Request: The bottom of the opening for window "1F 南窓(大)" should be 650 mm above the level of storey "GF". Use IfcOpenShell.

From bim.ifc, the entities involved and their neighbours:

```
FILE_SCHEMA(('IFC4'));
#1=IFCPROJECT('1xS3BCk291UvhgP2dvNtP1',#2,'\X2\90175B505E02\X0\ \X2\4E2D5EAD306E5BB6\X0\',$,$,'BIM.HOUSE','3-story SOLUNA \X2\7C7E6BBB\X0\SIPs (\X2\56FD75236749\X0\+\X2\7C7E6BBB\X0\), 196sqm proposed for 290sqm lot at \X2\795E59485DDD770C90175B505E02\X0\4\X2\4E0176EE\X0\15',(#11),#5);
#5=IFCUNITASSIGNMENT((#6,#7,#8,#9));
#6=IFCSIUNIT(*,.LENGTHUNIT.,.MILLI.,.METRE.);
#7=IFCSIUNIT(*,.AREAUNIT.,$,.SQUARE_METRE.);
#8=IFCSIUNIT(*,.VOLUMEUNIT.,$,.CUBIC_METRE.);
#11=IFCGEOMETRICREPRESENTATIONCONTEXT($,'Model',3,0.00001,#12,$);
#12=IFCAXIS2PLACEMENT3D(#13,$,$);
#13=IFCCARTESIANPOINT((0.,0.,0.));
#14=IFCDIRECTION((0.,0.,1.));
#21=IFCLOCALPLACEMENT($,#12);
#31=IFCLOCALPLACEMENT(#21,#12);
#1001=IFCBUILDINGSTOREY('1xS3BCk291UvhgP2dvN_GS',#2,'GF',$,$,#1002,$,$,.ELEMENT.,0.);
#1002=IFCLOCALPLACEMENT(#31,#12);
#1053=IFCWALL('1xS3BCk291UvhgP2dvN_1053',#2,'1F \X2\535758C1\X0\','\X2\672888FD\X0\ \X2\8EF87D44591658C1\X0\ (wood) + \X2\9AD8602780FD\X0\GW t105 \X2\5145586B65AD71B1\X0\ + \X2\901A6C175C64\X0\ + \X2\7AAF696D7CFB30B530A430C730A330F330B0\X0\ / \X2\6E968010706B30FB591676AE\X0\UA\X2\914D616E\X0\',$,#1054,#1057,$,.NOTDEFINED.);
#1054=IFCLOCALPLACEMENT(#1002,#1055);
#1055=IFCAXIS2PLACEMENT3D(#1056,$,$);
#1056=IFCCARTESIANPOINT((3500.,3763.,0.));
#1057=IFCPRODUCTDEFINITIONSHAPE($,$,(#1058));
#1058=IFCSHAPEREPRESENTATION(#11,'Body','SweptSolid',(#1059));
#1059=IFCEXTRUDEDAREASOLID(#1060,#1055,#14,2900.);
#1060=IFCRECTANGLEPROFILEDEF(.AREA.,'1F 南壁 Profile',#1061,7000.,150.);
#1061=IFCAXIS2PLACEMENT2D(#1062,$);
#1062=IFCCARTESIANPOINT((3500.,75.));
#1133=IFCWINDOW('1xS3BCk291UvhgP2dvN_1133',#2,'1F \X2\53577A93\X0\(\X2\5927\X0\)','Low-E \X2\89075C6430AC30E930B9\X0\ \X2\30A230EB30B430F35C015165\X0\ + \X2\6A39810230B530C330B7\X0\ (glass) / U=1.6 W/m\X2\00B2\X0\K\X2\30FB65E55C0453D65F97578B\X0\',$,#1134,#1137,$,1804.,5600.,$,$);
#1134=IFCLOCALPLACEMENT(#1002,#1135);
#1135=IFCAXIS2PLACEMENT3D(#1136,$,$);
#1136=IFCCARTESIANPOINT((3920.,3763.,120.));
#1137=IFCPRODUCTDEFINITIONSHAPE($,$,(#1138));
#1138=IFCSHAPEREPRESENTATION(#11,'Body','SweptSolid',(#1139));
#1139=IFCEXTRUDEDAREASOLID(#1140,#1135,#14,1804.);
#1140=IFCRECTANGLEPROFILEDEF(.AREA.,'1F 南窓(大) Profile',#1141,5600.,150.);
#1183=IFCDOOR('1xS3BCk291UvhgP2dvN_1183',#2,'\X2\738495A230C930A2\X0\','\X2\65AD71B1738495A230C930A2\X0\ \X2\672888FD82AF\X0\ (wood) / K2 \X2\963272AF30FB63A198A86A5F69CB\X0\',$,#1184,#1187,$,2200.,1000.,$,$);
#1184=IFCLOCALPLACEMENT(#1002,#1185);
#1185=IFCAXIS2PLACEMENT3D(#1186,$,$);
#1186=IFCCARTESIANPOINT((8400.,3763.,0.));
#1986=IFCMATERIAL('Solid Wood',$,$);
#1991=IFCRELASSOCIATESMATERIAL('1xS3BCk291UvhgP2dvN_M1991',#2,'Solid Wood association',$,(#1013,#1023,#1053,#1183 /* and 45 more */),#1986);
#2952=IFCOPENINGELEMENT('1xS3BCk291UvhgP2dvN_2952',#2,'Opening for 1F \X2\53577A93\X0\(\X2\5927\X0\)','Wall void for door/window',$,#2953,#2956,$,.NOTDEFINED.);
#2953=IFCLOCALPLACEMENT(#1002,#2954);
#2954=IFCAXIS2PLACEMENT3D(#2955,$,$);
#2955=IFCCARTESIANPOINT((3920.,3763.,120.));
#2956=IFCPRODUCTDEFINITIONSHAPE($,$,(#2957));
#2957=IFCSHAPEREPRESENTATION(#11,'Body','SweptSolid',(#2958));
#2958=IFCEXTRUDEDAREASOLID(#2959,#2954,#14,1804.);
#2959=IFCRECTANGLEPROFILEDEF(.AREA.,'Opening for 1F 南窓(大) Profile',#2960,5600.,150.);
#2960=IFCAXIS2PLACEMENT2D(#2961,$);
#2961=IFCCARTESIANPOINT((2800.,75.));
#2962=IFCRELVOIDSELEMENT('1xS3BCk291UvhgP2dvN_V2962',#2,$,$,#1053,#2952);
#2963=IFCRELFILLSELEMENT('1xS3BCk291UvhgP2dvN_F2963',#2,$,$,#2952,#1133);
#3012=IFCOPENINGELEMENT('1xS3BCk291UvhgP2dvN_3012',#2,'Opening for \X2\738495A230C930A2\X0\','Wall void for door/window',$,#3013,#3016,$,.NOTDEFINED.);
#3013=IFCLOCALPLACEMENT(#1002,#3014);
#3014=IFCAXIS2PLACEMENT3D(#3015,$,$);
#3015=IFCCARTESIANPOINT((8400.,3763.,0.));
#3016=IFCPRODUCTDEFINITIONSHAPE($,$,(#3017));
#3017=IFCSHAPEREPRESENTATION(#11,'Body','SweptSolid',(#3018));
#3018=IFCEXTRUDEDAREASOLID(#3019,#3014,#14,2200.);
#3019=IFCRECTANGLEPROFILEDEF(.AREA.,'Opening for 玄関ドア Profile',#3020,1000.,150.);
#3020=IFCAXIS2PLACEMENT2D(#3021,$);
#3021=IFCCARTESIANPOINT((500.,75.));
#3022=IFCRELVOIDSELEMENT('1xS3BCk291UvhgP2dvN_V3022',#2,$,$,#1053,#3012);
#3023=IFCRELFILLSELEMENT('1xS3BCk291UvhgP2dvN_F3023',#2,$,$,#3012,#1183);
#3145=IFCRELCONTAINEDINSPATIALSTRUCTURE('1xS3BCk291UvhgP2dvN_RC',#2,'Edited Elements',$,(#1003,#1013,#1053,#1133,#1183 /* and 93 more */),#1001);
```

```python
import numpy as np
import ifcopenshell
import ifcopenshell.api.geometry
import ifcopenshell.geom
import ifcopenshell.util.element
import ifcopenshell.util.placement
import ifcopenshell.util.shape
import ifcopenshell.util.unit

model = ifcopenshell.open("bim.ifc")
unit_scale = ifcopenshell.util.unit.calculate_unit_scale(model)

window = model.by_guid("1xS3BCk291UvhgP2dvN_1133")
opening = window.FillsVoids[0].RelatingOpeningElement
storey = ifcopenshell.util.element.get_container(window, ifc_class="IfcBuildingStorey")
level = ifcopenshell.util.placement.get_local_placement(storey.ObjectPlacement)[2, 3]

# The opening's origin need not be at the sill, so measure its lowest point.
shape = ifcopenshell.geom.create_shape(ifcopenshell.geom.settings(), opening)
bottom = ifcopenshell.util.shape.get_shape_bottom_elevation(shape, shape.geometry) / unit_scale
dz = level + 0.65 / unit_scale - bottom

shift = np.array([0.0, 0.0, dz])
# The window is not placed relative to its opening, so move both.
for product in (opening, window):
    matrix = ifcopenshell.util.placement.get_local_placement(product.ObjectPlacement)
    matrix[:3, 3] += shift
    ifcopenshell.api.geometry.edit_object_placement(model, product=product, matrix=matrix, is_si=False)

print(f"moved by {dz * unit_scale:+.3f} m")

model.write("bim_v2.ifc")
```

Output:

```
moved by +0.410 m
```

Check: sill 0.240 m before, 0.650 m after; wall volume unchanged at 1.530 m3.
